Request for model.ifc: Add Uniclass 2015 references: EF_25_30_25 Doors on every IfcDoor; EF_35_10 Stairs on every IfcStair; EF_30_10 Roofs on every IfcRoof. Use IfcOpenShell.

First a look at what the model holds.

```python
import ifcopenshell

model = ifcopenshell.open("model.ifc")
print(model.schema)
print("classifications:", [c.Name for c in model.by_type("IfcClassification")])
for ifc_class in ("IfcDoor", "IfcRoof", "IfcStair", "IfcWall", "IfcWindow"):
    print(ifc_class, len(model.by_type(ifc_class)))
```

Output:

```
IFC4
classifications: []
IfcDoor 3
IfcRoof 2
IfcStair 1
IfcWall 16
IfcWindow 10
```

```python
import ifcopenshell
import ifcopenshell.api.classification

model = ifcopenshell.open("model.ifc")

system = ifcopenshell.api.classification.add_classification(model, classification="Uniclass 2015")

codes = {
    "IfcDoor": ("EF_25_30_25", "Doors"),
    "IfcStair": ("EF_35_10", "Stairs"),
    "IfcRoof": ("EF_30_10", "Roofs"),
}
for ifc_class, (code, name) in codes.items():
    products = model.by_type(ifc_class)
    ifcopenshell.api.classification.add_reference(
        model, products=products, classification=system, identification=code, name=name
    )
    print(code, len(products))

model.write("model_edited.ifc")
```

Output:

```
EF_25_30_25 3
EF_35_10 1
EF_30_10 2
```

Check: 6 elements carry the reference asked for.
